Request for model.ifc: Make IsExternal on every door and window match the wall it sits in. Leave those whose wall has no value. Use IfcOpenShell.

First a look at what the model holds.

```python
import ifcopenshell
import ifcopenshell.util.element

model = ifcopenshell.open("model.ifc")
print(model.schema)
seen = {}
for e in model.by_type("IfcDoor") + model.by_type("IfcWindow"):
    if not e.FillsVoids:
        continue
    host = e.FillsVoids[0].RelatingOpeningElement.VoidsElements[0].RelatingBuildingElement
    own = ifcopenshell.util.element.get_pset(e, f"Pset_{e.is_a()[3:].removesuffix('StandardCase')}Common", "IsExternal")
    wall = ifcopenshell.util.element.get_pset(host, "Pset_WallCommon", "IsExternal")
    seen[e.is_a(), own, wall] = seen.get((e.is_a(), own, wall), 0) + 1
for (cls, own, wall), count in sorted(seen.items(), key=str):
    print(count, cls, "IsExternal:", own, "| host wall:", wall)
```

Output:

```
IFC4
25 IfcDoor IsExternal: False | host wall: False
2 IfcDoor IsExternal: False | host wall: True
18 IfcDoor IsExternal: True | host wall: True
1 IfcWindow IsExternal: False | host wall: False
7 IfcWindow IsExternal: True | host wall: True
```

```python
import ifcopenshell
import ifcopenshell.api.pset
import ifcopenshell.util.element

model = ifcopenshell.open("model.ifc")

count = 0
for ifc_class, pset_name in (("IfcDoor", "Pset_DoorCommon"), ("IfcWindow", "Pset_WindowCommon")):
    for e in model.by_type(ifc_class):
        if not e.FillsVoids:
            continue
        host = e.FillsVoids[0].RelatingOpeningElement.VoidsElements[0].RelatingBuildingElement
        external = ifcopenshell.util.element.get_pset(host, "Pset_WallCommon", "IsExternal")
        if external is None or ifcopenshell.util.element.get_pset(e, pset_name, "IsExternal") == external:
            continue
        pset = ifcopenshell.api.pset.add_pset(model, product=e, name=pset_name)
        ifcopenshell.api.pset.edit_pset(model, pset=pset, properties={"IsExternal": external})
        count += 1

print(count, "updated")

model.write("model_v2.ifc")
```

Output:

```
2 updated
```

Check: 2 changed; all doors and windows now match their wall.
